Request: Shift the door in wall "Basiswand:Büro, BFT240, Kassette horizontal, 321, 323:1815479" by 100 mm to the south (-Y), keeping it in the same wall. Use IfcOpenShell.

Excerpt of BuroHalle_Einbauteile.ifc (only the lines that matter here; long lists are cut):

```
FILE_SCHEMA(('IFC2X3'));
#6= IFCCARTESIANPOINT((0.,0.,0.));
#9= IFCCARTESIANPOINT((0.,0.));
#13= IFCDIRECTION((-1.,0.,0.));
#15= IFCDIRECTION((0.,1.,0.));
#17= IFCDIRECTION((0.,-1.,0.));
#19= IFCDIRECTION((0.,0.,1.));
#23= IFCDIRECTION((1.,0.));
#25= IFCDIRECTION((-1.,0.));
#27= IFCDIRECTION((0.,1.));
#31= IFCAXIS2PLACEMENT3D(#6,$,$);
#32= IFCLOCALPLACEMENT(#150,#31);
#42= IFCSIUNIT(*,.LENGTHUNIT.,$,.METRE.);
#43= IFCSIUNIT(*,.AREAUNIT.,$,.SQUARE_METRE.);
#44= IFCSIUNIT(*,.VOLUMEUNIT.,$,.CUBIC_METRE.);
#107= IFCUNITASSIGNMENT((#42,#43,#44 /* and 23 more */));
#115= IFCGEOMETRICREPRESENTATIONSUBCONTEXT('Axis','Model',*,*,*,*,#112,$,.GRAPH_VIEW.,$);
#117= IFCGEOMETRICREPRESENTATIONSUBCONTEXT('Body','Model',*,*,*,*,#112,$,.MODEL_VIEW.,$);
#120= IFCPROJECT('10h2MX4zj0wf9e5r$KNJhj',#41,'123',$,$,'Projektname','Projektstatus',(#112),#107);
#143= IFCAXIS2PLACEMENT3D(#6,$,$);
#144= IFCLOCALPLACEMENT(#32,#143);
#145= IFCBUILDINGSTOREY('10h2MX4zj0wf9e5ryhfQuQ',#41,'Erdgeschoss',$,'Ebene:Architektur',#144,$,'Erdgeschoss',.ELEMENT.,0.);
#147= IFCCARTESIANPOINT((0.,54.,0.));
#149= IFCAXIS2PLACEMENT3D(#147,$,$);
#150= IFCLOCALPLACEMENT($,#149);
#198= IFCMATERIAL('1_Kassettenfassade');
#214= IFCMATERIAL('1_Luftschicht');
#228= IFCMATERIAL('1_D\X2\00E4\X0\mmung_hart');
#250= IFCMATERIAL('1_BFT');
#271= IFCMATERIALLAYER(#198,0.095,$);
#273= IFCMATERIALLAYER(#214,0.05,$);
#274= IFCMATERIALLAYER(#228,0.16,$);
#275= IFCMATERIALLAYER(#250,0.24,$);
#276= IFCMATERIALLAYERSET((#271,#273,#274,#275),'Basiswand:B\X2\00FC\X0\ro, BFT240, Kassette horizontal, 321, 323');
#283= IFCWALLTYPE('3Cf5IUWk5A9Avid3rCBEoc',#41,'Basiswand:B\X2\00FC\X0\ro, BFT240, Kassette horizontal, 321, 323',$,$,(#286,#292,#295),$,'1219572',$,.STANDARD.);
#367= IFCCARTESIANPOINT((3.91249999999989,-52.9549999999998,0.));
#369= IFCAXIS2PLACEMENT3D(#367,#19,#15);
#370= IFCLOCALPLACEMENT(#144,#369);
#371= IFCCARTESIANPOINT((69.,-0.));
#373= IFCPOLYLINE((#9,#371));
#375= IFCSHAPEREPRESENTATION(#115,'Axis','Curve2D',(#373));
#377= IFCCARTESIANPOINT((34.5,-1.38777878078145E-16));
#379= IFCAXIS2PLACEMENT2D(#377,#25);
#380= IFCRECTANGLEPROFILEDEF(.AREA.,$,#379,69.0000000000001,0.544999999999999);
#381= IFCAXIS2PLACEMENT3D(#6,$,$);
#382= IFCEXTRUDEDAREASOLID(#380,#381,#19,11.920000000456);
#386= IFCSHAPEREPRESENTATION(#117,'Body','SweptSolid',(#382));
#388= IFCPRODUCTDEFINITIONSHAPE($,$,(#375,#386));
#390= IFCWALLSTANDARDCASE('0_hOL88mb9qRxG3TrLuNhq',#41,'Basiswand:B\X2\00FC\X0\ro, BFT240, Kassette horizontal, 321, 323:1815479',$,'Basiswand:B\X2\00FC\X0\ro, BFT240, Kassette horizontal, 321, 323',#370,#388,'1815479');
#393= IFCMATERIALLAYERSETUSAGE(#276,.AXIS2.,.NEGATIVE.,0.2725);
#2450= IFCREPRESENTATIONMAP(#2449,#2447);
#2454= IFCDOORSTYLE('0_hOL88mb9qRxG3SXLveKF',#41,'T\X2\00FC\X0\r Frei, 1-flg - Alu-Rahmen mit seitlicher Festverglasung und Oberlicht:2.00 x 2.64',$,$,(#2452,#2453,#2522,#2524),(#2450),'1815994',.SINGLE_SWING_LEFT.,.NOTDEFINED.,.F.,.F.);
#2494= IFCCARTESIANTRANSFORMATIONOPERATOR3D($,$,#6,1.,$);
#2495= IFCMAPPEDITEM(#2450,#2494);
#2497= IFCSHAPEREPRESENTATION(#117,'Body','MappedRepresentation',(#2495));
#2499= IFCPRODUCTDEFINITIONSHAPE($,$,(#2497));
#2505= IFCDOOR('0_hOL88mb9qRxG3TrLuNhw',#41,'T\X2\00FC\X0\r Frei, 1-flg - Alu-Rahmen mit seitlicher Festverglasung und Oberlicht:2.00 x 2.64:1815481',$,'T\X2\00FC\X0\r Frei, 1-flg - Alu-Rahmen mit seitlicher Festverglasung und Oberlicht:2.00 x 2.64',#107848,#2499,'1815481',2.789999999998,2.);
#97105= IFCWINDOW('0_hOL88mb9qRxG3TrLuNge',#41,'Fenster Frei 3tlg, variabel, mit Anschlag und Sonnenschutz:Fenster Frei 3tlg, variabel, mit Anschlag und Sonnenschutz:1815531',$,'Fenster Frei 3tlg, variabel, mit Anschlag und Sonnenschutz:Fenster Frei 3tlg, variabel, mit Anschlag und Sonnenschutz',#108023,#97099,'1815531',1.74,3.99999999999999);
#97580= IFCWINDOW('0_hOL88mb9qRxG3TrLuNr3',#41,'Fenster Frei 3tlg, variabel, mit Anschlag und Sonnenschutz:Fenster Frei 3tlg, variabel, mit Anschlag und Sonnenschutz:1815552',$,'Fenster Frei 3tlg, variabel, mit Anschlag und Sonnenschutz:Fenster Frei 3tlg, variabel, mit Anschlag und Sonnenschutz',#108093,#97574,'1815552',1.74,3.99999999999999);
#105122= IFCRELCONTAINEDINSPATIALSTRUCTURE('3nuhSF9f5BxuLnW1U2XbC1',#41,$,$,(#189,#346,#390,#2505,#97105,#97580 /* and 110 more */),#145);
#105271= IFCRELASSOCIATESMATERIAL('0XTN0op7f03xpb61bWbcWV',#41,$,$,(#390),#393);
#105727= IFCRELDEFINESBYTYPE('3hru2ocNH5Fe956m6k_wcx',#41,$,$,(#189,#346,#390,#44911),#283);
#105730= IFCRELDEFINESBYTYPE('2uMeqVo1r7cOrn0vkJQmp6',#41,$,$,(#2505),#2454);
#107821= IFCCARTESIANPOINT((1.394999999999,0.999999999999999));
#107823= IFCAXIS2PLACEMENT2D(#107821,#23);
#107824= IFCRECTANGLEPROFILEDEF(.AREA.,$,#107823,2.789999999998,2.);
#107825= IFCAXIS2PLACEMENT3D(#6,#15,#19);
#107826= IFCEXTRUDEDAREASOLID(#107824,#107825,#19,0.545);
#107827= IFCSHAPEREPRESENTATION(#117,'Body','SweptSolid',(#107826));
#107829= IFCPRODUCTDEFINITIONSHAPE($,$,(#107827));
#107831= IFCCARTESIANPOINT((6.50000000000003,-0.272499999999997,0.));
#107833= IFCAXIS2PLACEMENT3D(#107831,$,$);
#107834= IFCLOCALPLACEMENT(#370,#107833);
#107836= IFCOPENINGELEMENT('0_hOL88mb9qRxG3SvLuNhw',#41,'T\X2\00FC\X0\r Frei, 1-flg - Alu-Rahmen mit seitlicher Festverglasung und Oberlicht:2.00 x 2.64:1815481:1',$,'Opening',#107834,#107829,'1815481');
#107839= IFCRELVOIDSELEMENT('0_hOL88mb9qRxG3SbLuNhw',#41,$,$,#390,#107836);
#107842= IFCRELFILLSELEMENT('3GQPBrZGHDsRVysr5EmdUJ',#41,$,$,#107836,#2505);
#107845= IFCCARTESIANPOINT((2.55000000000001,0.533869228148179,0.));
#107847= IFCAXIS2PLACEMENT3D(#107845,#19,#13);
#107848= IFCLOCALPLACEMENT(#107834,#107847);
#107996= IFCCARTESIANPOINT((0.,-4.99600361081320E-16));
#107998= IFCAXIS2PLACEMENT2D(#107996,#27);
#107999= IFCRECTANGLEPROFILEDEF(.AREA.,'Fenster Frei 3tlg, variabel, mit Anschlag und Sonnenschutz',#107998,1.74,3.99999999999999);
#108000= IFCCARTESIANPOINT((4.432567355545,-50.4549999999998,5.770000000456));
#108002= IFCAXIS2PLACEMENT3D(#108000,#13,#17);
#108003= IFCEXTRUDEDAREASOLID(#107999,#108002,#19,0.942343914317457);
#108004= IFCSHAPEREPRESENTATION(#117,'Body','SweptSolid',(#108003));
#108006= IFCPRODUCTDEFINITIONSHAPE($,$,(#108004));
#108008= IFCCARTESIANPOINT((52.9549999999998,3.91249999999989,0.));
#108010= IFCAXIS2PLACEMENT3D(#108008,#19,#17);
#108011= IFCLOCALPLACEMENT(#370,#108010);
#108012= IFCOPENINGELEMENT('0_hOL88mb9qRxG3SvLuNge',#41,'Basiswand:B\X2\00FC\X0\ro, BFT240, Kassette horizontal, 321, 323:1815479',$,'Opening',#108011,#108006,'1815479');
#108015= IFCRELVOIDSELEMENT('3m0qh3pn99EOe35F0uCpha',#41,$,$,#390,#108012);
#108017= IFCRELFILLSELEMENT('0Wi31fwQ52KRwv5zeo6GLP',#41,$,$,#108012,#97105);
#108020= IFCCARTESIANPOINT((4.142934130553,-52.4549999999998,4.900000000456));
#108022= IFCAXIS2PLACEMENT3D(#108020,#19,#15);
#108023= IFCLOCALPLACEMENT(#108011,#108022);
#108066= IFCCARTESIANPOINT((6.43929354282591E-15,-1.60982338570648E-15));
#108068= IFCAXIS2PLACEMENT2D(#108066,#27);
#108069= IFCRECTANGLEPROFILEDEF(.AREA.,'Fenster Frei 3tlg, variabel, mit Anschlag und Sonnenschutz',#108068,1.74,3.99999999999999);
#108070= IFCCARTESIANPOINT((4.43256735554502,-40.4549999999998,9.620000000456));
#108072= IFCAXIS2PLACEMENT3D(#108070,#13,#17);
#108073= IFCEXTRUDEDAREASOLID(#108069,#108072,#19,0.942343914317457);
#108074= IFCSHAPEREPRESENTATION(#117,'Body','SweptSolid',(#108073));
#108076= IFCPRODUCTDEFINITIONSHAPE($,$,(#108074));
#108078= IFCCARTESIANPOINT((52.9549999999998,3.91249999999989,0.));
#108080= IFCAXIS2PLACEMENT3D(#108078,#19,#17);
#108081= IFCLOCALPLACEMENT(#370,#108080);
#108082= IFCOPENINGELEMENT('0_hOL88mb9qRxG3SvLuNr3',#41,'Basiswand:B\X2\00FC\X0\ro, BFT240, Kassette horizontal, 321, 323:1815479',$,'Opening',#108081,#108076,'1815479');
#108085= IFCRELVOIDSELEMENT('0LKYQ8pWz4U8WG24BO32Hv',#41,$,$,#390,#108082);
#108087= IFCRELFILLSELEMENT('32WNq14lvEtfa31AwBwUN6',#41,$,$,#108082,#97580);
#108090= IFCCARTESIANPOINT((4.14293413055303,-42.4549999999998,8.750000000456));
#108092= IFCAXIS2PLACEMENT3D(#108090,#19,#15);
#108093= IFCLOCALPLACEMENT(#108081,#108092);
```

```python
import ifcopenshell
import ifcopenshell.api.geometry
import ifcopenshell.util.placement
import ifcopenshell.util.unit

model = ifcopenshell.open("BuroHalle_Einbauteile.ifc")
unit_scale = ifcopenshell.util.unit.calculate_unit_scale(model)

door = model.by_guid("0_hOL88mb9qRxG3TrLuNhw")
opening = door.FillsVoids[0].RelatingOpeningElement
wall = opening.VoidsElements[0].RelatingBuildingElement

wall_matrix = ifcopenshell.util.placement.get_local_placement(wall.ObjectPlacement)
shift = wall_matrix[:3, 0] * -0.1 / unit_scale
before = ifcopenshell.util.placement.get_local_placement(door.ObjectPlacement)[:3, 3].copy()

# The door is placed relative to its opening, so it follows when the opening moves.
matrix = ifcopenshell.util.placement.get_local_placement(opening.ObjectPlacement)
matrix[:3, 3] += shift
ifcopenshell.api.geometry.edit_object_placement(
    model, product=opening, matrix=matrix, is_si=False, should_transform_children=True
)

after = ifcopenshell.util.placement.get_local_placement(door.ObjectPlacement)[:3, 3]
print("door moved by", (after - before).round(3) + 0.0)

model.write("BuroHalle_Einbauteile_v2.ifc")
```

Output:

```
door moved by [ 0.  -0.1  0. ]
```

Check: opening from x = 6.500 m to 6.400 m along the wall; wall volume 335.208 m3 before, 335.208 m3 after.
